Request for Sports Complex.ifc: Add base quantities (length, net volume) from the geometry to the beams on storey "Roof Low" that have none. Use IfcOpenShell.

First a look at what the model holds.

```python
import ifcopenshell
import ifcopenshell.util.element
import ifcopenshell.util.unit

model = ifcopenshell.open("Sports Complex.ifc")
print(model.schema)
for unit_type in ("LENGTHUNIT", "AREAUNIT", "VOLUMEUNIT"):
    print(unit_type, ifcopenshell.util.unit.calculate_unit_scale(model, unit_type))
storey = next(s for s in model.by_type("IfcBuildingStorey") if s.Name == "Roof Low")
beams = [e for e in ifcopenshell.util.element.get_decomposition(storey) if e.is_a("IfcBeam")]
for e in sorted(beams, key=lambda e: e.id()):
    print(e.id(), e.is_a(), e.Name, list(ifcopenshell.util.element.get_psets(e, qtos_only=True)), sep=" | ")
```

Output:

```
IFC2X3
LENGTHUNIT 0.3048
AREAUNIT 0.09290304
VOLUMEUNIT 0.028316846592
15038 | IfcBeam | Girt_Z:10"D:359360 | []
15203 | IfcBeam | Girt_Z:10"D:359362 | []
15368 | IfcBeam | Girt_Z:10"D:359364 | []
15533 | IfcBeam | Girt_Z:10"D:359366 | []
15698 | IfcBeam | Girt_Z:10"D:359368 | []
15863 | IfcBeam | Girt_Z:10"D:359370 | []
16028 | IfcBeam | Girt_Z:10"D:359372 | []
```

```python
import ifcopenshell
import ifcopenshell.api.pset
import ifcopenshell.geom
import ifcopenshell.util.element
import ifcopenshell.util.shape
import ifcopenshell.util.unit

model = ifcopenshell.open("Sports Complex.ifc")
unit_scale = ifcopenshell.util.unit.calculate_unit_scale(model)
volume_scale = ifcopenshell.util.unit.calculate_unit_scale(model, "VOLUMEUNIT")
settings = ifcopenshell.geom.settings()

storey = next(s for s in model.by_type("IfcBuildingStorey") if s.Name == "Roof Low")
beams = [e for e in ifcopenshell.util.element.get_decomposition(storey) if e.is_a("IfcBeam")]

for e in sorted(beams, key=lambda e: e.id()):
    if ifcopenshell.util.element.get_psets(e, qtos_only=True, should_inherit=False):
        continue
    # Geometry comes back in metres, in the element's own axes.
    shape = ifcopenshell.geom.create_shape(settings, e)
    values = {
        "Length": ifcopenshell.util.shape.get_max_xyz(shape.geometry) / unit_scale,
        "NetVolume": ifcopenshell.util.shape.get_volume(shape.geometry) / volume_scale,
    }
    qto = ifcopenshell.api.pset.add_qto(model, product=e, name="BaseQuantities")
    ifcopenshell.api.pset.edit_qto(model, qto=qto, properties=values)
    print(e.id(), {k: round(v, 3) for k, v in values.items()})

model.write("Sports Complex_rev.ifc")
```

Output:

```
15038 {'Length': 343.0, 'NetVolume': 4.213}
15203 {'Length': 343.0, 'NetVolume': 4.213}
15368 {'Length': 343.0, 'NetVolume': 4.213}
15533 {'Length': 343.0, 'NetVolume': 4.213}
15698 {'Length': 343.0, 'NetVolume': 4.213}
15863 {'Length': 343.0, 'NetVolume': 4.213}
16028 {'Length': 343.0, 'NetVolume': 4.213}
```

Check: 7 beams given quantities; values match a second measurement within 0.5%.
